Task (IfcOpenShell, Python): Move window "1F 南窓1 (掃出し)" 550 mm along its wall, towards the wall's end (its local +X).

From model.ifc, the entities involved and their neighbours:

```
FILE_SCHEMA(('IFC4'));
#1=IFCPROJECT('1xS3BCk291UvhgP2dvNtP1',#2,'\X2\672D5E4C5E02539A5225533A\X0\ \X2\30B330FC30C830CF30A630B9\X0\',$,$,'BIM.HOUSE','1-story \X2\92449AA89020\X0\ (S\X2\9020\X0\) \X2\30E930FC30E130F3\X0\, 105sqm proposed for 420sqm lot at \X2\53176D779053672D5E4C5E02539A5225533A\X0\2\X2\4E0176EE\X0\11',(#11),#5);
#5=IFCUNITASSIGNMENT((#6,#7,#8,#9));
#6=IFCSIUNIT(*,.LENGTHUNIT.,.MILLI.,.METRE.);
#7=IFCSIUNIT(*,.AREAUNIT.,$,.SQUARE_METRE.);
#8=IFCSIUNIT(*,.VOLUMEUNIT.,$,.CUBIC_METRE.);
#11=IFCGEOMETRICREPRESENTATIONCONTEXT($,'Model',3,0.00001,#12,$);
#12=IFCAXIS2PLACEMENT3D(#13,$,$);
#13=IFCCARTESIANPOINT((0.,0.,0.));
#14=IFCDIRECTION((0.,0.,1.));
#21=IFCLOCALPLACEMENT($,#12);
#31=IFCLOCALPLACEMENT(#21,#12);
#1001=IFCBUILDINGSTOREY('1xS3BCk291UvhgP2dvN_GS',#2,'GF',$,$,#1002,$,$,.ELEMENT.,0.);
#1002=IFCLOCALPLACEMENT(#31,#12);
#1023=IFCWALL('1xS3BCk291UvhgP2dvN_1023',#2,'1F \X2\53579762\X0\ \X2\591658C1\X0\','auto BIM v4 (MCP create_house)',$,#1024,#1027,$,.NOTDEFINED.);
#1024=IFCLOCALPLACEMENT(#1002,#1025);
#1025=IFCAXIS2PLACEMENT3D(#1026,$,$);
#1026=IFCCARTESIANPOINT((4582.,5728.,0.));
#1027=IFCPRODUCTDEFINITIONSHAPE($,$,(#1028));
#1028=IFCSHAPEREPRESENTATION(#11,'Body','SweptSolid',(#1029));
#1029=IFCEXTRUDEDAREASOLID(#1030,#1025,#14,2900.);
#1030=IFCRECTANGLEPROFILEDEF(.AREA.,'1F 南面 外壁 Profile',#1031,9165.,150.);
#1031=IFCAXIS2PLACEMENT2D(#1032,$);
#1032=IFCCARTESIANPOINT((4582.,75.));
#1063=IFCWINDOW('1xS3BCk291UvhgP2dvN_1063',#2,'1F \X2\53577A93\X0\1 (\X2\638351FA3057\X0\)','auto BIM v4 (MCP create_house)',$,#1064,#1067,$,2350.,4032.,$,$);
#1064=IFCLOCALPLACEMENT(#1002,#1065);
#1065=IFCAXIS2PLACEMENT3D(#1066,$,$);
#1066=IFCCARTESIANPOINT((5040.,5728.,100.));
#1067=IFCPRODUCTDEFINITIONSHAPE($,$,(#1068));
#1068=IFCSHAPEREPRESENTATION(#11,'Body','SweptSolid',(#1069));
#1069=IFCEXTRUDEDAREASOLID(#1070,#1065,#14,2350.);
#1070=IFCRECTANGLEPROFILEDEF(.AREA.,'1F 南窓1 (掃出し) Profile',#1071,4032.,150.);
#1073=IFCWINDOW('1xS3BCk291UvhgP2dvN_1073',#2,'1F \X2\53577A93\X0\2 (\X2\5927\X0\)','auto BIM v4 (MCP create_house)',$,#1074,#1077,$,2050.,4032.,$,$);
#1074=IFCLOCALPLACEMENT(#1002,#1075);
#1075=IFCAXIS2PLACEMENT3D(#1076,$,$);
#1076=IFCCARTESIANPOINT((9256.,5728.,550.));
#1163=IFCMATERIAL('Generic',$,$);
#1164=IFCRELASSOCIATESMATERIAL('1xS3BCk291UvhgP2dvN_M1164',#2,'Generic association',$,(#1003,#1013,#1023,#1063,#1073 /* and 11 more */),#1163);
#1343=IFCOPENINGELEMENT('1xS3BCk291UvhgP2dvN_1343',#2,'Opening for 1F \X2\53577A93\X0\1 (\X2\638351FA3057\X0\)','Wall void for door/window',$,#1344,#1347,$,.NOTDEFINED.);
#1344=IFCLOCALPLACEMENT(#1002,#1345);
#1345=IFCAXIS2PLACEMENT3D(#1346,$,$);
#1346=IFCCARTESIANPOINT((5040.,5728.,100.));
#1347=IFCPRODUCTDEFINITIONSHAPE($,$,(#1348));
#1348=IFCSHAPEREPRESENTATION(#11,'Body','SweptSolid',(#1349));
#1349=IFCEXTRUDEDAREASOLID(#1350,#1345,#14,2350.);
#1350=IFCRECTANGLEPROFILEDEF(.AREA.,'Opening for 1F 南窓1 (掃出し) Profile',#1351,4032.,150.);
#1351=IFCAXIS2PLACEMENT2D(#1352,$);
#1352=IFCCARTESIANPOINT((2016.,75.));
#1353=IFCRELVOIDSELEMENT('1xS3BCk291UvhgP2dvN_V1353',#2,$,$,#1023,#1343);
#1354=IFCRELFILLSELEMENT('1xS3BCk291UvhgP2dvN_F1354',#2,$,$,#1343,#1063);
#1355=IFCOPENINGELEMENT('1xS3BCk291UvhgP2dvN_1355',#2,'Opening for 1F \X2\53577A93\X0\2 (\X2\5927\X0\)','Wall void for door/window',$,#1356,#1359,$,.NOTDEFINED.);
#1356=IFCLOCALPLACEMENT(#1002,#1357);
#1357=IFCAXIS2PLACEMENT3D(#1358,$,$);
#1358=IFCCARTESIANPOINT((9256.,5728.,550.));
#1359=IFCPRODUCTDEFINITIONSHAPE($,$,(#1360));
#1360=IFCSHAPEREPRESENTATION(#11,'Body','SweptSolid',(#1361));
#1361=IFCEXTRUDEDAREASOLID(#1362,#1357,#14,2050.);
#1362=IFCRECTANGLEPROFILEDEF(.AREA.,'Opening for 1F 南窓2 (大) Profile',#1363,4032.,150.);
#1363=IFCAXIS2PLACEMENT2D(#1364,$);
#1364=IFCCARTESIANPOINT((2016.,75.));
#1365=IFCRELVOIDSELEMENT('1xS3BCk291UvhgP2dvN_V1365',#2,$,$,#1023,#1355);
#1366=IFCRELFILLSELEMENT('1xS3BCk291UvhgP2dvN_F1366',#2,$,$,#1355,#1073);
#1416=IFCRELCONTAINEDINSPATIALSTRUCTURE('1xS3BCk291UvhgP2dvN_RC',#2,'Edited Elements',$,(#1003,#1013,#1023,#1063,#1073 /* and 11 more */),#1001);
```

```python
import ifcopenshell
import ifcopenshell.api.geometry
import ifcopenshell.util.placement

model = ifcopenshell.open("model.ifc")

window = model.by_id(1063)
opening = window.FillsVoids[0].RelatingOpeningElement
wall = opening.VoidsElements[0].RelatingBuildingElement

wall_matrix = ifcopenshell.util.placement.get_local_placement(wall.ObjectPlacement)
shift = wall_matrix[:3, 0] * 550.0
before = ifcopenshell.util.placement.get_local_placement(window.ObjectPlacement)[:3, 3].copy()

# The window is not placed relative to its opening, so move both.
for product in (opening, window):
    matrix = ifcopenshell.util.placement.get_local_placement(product.ObjectPlacement)
    matrix[:3, 3] += shift
    ifcopenshell.api.geometry.edit_object_placement(model, product=product, matrix=matrix, is_si=False)

after = ifcopenshell.util.placement.get_local_placement(window.ObjectPlacement)[:3, 3]
print("window moved by", (after - before).round(3) + 0.0)

model.write("model_edited.ifc")
```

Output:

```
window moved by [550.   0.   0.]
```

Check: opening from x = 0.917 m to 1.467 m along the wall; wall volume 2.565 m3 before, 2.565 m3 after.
